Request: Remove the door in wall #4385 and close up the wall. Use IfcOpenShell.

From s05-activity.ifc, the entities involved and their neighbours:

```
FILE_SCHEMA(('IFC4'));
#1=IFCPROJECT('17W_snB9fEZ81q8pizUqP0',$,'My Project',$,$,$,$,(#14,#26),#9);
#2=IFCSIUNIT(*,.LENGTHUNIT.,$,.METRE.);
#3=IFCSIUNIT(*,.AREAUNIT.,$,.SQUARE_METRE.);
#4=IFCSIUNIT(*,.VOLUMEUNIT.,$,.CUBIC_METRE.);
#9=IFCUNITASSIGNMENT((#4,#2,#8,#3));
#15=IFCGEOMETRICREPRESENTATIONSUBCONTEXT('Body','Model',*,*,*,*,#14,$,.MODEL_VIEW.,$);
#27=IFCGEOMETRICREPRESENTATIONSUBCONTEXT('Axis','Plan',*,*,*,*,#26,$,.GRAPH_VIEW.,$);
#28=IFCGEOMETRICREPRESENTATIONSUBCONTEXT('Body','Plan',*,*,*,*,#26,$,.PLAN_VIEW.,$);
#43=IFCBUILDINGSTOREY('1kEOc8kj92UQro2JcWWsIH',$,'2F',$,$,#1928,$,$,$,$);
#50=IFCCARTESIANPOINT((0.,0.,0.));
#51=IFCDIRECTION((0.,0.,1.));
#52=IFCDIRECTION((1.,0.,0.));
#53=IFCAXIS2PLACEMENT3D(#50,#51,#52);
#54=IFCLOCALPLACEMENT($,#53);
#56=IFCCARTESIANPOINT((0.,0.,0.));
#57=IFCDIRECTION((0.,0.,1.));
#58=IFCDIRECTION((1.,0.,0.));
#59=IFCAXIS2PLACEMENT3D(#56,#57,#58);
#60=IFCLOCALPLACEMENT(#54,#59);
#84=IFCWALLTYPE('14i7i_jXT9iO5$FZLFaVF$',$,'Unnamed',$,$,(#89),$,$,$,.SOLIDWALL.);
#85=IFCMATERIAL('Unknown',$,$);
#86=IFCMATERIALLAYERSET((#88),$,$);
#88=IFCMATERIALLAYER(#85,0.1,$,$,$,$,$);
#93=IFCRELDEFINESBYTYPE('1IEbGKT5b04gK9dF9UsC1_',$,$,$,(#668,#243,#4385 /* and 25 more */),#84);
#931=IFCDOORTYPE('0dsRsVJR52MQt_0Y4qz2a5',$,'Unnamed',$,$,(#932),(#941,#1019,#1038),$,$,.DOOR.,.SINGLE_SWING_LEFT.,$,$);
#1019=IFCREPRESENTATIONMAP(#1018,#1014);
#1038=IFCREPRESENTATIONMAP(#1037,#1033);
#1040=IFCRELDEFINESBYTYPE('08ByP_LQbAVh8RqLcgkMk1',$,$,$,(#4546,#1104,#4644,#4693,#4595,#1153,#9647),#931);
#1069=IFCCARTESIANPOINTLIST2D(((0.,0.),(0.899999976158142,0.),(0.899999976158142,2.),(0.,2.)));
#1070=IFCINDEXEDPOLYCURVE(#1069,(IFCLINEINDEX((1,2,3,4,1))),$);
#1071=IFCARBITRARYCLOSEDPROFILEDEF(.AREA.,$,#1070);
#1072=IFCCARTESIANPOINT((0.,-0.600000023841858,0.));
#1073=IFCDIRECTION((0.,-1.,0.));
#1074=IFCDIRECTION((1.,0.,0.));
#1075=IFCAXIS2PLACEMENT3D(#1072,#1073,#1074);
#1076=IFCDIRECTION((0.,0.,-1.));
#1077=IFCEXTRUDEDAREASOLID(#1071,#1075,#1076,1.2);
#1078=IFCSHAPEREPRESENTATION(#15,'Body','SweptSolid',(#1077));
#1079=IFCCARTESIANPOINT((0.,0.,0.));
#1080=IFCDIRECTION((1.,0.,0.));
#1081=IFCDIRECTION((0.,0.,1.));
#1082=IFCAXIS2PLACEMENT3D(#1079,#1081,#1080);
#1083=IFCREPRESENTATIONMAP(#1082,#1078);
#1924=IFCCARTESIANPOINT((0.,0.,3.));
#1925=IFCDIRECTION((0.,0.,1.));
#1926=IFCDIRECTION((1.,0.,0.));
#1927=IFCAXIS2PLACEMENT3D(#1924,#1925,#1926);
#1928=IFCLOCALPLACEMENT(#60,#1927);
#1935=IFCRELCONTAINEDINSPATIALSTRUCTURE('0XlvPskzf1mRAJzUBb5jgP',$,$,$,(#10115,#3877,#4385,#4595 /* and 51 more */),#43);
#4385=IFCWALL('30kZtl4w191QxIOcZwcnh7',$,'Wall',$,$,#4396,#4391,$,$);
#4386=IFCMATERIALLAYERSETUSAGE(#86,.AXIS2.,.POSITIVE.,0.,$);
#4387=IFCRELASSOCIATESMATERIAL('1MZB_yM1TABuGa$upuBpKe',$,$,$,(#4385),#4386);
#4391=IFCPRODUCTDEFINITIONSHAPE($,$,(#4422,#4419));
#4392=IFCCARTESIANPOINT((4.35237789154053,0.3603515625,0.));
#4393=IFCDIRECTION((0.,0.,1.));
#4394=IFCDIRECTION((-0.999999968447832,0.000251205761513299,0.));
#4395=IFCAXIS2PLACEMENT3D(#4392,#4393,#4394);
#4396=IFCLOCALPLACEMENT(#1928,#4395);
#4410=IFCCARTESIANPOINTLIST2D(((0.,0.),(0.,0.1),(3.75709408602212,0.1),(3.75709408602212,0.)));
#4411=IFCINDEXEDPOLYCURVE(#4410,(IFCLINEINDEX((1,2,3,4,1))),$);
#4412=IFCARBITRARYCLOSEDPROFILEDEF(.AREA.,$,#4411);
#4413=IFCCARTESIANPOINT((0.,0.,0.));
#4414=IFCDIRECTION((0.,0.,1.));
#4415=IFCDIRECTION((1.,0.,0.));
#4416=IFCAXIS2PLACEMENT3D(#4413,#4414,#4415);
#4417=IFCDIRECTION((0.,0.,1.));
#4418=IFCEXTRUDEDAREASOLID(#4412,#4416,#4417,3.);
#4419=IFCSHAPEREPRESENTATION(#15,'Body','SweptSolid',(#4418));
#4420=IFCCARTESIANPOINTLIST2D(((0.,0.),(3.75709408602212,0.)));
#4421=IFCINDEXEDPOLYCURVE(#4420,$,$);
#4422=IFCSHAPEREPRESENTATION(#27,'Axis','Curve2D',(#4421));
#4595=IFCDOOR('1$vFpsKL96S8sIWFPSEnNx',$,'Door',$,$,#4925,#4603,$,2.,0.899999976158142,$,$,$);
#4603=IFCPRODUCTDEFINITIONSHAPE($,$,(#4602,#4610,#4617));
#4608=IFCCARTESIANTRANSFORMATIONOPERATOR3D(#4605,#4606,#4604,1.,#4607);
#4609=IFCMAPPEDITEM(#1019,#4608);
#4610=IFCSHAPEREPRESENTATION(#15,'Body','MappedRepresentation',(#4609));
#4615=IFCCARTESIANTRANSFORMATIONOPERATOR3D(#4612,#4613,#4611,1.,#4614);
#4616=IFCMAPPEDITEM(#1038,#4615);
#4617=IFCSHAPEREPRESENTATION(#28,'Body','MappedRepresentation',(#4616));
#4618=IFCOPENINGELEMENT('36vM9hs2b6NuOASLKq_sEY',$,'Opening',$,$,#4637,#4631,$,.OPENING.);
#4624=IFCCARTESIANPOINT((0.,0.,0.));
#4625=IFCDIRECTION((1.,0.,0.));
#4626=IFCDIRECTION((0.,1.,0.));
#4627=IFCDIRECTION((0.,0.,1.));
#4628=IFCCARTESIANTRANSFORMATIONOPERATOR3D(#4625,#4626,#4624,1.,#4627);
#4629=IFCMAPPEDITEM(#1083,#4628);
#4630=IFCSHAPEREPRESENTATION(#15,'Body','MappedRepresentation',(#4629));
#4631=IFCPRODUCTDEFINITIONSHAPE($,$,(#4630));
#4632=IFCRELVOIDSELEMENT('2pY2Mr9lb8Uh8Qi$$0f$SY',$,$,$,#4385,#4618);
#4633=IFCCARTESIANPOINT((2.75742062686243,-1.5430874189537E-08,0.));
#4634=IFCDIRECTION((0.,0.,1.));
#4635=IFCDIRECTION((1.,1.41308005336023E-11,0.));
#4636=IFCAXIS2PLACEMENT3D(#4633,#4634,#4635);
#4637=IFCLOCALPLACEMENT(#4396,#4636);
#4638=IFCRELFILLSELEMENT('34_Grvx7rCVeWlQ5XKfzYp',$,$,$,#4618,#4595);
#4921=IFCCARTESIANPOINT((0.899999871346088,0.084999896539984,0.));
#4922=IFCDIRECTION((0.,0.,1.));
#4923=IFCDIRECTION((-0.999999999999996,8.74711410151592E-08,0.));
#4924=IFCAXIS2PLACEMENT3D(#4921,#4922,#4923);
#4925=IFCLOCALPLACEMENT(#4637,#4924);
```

```python
import ifcopenshell
import ifcopenshell.api.feature
import ifcopenshell.api.root
import ifcopenshell.geom
import ifcopenshell.util.shape

model = ifcopenshell.open("s05-activity.ifc")
settings = ifcopenshell.geom.settings()


def volume(element):
    """Net volume in cubic metres, openings subtracted."""
    shape = ifcopenshell.geom.create_shape(settings, element)
    return ifcopenshell.util.shape.get_volume(shape.geometry)


door = model.by_guid("1$vFpsKL96S8sIWFPSEnNx")
opening = door.FillsVoids[0].RelatingOpeningElement
wall = opening.VoidsElements[0].RelatingBuildingElement
before = volume(wall)

ifcopenshell.api.root.remove_product(model, product=door)
ifcopenshell.api.feature.remove_feature(model, feature=opening)

after = volume(wall)

print(f"wall volume {before:.3f} -> {after:.3f} m3")

model.write("s05-activity-out.ifc")
```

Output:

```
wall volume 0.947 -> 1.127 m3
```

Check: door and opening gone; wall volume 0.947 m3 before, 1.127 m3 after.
